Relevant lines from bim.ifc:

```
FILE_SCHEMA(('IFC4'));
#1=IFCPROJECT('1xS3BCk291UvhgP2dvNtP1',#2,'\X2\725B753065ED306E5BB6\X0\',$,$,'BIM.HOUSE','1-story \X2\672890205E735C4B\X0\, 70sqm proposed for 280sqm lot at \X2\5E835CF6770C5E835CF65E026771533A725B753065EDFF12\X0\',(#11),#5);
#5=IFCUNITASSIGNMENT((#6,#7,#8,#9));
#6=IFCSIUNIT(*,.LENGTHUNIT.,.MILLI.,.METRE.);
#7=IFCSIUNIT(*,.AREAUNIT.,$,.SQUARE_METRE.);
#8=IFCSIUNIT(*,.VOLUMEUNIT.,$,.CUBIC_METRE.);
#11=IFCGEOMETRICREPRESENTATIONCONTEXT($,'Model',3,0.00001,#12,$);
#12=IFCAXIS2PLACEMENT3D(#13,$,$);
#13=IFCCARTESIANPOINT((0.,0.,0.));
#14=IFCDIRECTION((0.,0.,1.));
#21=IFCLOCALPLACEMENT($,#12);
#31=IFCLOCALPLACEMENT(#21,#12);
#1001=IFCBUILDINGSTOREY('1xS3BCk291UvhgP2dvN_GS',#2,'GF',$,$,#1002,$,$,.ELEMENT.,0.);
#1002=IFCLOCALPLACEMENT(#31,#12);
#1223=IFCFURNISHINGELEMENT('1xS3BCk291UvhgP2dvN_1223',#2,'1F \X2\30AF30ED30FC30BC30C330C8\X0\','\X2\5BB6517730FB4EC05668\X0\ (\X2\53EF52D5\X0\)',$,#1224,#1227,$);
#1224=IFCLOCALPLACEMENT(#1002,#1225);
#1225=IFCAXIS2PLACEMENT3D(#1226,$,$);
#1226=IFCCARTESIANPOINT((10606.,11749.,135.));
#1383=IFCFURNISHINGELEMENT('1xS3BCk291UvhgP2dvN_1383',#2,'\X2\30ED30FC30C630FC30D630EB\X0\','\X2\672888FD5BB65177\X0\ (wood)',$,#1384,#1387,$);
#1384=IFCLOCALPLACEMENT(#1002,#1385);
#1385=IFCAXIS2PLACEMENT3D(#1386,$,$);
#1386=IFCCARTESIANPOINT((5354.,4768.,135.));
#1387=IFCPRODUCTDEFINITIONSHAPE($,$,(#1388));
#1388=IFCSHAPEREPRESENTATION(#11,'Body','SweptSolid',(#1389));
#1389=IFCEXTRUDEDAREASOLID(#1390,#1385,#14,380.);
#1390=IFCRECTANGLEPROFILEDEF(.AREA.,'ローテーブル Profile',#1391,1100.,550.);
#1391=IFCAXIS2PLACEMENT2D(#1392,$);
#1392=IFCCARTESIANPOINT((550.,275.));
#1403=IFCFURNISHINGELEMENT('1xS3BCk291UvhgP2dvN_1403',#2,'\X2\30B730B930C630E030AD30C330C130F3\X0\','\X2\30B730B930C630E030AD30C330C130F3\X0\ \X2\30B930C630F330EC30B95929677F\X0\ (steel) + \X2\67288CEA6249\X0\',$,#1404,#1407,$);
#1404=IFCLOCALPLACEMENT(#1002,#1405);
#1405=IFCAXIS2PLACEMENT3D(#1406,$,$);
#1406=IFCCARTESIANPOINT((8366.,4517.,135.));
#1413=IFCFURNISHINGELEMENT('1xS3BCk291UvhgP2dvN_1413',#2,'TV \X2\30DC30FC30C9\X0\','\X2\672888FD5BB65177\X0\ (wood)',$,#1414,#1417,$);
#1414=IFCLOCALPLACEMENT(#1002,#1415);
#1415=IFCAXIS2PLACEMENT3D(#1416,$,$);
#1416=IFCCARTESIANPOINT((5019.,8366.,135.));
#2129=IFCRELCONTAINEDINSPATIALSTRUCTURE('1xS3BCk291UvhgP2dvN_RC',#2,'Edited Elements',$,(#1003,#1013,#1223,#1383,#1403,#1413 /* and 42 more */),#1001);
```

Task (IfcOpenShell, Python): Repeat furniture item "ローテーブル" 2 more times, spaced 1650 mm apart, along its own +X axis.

```python
import ifcopenshell
import ifcopenshell.api.geometry
import ifcopenshell.api.root
import ifcopenshell.util.element
import ifcopenshell.util.placement
import ifcopenshell.util.unit

model = ifcopenshell.open("bim.ifc")
unit_scale = ifcopenshell.util.unit.calculate_unit_scale(model)


def reuse_history(source, copy):
    """copy_class also copies each property set's owner history, people and application; keep the originals."""
    for rel in copy.IsDefinedBy:
        if rel.is_a("IfcRelDefinesByProperties") and (history := rel.RelatingPropertyDefinition.OwnerHistory):
            rel.RelatingPropertyDefinition.OwnerHistory = source.OwnerHistory
            ifcopenshell.util.element.remove_deep2(model, history)


source = model.by_guid("1xS3BCk291UvhgP2dvN_1383")
base = ifcopenshell.util.placement.get_local_placement(source.ObjectPlacement)
step = base[:3, 0] * 1.65 / unit_scale

for i in range(1, 3):
    copy = ifcopenshell.api.root.copy_class(model, product=source)
    copy.Representation = ifcopenshell.util.element.copy_deep(
        model, source.Representation, exclude=["IfcGeometricRepresentationContext", "IfcRepresentationMap"]
    )
    reuse_history(source, copy)
    matrix = base.copy()
    matrix[:3, 3] += i * step
    print("added at", matrix[:3, 3].round(3) + 0.0)
    ifcopenshell.api.geometry.edit_object_placement(model, product=copy, matrix=matrix, is_si=False)

model.write("bim_rev.ifc")
```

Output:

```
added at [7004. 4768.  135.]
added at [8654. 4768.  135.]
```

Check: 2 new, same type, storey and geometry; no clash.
